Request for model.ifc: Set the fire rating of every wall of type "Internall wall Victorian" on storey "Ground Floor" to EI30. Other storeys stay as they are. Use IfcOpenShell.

First a look at what the model holds.

```python
import ifcopenshell
import ifcopenshell.util.element

model = ifcopenshell.open("model.ifc")
print(model.schema)
storey = next(s for s in model.by_type("IfcBuildingStorey") if s.Name == "Ground Floor")
walls = [e for e in ifcopenshell.util.element.get_decomposition(storey) if e.is_a("IfcWall")]
seen = {}
for e in walls:
    element_type = ifcopenshell.util.element.get_type(e)
    key = (element_type.Name if element_type != e and element_type else None, ifcopenshell.util.element.get_pset(e, "Pset_WallCommon", "FireRating"))
    seen[key] = seen.get(key, 0) + 1
for (name, value), count in sorted(seen.items(), key=str):
    print(count, "x", name, "|", value)
```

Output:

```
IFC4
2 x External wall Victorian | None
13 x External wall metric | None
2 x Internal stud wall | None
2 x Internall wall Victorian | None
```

```python
import ifcopenshell
import ifcopenshell.api.pset
import ifcopenshell.util.element

model = ifcopenshell.open("model.ifc")

storey = next(s for s in model.by_type("IfcBuildingStorey") if s.Name == "Ground Floor")
walls = [e for e in ifcopenshell.util.element.get_decomposition(storey) if e.is_a("IfcWall")]

count = 0
for e in walls:
    element_type = ifcopenshell.util.element.get_type(e)
    if element_type in (None, e) or element_type.Name != "Internall wall Victorian":
        continue
    # add_pset returns the element's existing set when there is one.
    pset = ifcopenshell.api.pset.add_pset(model, product=e, name="Pset_WallCommon")
    ifcopenshell.api.pset.edit_pset(model, pset=pset, properties={"FireRating": "EI30"})
    count += 1

print(count, "walls updated")

model.write("model_rev.ifc")
```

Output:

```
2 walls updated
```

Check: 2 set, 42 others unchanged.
